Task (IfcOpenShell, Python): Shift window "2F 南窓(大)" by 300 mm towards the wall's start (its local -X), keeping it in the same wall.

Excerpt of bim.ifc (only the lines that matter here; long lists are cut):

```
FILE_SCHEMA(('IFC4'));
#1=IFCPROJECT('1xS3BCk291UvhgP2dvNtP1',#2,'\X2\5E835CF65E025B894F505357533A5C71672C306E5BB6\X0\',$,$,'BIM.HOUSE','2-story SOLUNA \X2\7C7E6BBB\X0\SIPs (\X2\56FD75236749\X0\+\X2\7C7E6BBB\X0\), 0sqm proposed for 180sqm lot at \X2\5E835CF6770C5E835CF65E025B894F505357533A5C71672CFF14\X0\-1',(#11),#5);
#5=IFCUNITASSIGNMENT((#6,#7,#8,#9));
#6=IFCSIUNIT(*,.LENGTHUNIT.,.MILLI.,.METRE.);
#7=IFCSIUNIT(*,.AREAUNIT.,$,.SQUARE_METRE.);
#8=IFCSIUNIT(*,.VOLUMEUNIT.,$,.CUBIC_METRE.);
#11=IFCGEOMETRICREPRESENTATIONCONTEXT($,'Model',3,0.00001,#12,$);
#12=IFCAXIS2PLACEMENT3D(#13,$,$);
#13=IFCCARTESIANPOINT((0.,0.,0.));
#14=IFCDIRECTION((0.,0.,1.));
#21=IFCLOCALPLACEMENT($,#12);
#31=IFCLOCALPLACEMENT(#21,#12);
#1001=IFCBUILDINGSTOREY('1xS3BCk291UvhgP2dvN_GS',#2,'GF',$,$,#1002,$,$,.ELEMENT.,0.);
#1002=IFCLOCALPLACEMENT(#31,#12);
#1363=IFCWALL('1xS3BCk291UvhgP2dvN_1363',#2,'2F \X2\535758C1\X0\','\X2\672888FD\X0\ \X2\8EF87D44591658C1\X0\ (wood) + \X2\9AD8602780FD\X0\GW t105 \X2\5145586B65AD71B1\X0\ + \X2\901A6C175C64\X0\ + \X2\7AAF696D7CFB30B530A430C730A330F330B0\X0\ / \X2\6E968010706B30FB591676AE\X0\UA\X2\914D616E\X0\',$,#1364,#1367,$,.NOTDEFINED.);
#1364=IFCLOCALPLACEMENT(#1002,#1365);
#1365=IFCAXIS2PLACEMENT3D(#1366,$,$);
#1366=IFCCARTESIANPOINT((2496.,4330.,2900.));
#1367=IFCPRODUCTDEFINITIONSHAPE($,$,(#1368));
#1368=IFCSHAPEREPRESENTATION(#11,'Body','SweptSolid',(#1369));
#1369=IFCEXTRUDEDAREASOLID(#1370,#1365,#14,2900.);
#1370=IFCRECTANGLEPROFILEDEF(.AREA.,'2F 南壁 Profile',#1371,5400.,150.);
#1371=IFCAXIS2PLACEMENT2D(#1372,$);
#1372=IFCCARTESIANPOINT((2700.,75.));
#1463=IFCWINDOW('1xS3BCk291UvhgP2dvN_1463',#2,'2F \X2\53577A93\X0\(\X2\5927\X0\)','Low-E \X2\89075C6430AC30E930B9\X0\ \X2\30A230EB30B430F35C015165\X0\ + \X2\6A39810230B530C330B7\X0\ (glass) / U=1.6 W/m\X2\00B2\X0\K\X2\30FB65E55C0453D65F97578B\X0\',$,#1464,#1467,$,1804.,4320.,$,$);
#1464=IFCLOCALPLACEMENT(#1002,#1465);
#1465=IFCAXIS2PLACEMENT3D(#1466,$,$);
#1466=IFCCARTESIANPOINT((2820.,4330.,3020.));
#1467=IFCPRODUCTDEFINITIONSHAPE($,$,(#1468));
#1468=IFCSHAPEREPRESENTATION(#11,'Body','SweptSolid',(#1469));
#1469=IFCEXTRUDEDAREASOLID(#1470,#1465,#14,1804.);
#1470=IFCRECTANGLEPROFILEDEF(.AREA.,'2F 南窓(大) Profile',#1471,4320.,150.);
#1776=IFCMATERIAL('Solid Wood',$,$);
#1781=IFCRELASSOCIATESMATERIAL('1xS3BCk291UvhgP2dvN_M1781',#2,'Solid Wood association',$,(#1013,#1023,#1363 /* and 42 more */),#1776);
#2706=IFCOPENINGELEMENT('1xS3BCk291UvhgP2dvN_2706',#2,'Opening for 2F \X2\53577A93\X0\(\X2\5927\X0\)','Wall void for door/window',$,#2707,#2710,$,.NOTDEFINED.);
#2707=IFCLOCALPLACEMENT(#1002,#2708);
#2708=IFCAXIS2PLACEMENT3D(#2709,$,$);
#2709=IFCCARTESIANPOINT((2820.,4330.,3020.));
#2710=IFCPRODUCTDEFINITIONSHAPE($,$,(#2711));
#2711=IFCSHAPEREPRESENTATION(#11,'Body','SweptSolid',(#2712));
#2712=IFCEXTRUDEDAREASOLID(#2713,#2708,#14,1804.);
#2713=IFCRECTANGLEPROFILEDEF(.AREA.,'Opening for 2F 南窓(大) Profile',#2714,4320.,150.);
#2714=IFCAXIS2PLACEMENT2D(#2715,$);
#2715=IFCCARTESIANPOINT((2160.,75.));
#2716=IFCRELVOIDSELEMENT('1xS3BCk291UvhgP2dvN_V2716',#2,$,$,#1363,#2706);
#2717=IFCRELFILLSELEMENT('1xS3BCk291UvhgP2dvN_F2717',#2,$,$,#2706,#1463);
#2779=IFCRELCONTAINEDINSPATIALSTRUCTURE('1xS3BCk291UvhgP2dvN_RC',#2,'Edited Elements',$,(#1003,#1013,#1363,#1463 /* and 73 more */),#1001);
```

```python
import ifcopenshell
import ifcopenshell.api.geometry
import ifcopenshell.util.placement
import ifcopenshell.util.unit

model = ifcopenshell.open("bim.ifc")
unit_scale = ifcopenshell.util.unit.calculate_unit_scale(model)

window = model.by_id(1463)
opening = window.FillsVoids[0].RelatingOpeningElement
wall = opening.VoidsElements[0].RelatingBuildingElement

wall_matrix = ifcopenshell.util.placement.get_local_placement(wall.ObjectPlacement)
shift = wall_matrix[:3, 0] * -0.3 / unit_scale
before = ifcopenshell.util.placement.get_local_placement(window.ObjectPlacement)[:3, 3].copy()

# The window is not placed relative to its opening, so move both.
for product in (opening, window):
    matrix = ifcopenshell.util.placement.get_local_placement(product.ObjectPlacement)
    matrix[:3, 3] += shift
    ifcopenshell.api.geometry.edit_object_placement(model, product=product, matrix=matrix, is_si=False)

after = ifcopenshell.util.placement.get_local_placement(window.ObjectPlacement)[:3, 3]
print("window moved by", (after - before).round(3) + 0.0)

model.write("bim_rev.ifc")
```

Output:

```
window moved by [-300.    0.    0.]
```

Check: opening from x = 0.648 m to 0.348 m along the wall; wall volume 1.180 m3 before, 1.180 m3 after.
